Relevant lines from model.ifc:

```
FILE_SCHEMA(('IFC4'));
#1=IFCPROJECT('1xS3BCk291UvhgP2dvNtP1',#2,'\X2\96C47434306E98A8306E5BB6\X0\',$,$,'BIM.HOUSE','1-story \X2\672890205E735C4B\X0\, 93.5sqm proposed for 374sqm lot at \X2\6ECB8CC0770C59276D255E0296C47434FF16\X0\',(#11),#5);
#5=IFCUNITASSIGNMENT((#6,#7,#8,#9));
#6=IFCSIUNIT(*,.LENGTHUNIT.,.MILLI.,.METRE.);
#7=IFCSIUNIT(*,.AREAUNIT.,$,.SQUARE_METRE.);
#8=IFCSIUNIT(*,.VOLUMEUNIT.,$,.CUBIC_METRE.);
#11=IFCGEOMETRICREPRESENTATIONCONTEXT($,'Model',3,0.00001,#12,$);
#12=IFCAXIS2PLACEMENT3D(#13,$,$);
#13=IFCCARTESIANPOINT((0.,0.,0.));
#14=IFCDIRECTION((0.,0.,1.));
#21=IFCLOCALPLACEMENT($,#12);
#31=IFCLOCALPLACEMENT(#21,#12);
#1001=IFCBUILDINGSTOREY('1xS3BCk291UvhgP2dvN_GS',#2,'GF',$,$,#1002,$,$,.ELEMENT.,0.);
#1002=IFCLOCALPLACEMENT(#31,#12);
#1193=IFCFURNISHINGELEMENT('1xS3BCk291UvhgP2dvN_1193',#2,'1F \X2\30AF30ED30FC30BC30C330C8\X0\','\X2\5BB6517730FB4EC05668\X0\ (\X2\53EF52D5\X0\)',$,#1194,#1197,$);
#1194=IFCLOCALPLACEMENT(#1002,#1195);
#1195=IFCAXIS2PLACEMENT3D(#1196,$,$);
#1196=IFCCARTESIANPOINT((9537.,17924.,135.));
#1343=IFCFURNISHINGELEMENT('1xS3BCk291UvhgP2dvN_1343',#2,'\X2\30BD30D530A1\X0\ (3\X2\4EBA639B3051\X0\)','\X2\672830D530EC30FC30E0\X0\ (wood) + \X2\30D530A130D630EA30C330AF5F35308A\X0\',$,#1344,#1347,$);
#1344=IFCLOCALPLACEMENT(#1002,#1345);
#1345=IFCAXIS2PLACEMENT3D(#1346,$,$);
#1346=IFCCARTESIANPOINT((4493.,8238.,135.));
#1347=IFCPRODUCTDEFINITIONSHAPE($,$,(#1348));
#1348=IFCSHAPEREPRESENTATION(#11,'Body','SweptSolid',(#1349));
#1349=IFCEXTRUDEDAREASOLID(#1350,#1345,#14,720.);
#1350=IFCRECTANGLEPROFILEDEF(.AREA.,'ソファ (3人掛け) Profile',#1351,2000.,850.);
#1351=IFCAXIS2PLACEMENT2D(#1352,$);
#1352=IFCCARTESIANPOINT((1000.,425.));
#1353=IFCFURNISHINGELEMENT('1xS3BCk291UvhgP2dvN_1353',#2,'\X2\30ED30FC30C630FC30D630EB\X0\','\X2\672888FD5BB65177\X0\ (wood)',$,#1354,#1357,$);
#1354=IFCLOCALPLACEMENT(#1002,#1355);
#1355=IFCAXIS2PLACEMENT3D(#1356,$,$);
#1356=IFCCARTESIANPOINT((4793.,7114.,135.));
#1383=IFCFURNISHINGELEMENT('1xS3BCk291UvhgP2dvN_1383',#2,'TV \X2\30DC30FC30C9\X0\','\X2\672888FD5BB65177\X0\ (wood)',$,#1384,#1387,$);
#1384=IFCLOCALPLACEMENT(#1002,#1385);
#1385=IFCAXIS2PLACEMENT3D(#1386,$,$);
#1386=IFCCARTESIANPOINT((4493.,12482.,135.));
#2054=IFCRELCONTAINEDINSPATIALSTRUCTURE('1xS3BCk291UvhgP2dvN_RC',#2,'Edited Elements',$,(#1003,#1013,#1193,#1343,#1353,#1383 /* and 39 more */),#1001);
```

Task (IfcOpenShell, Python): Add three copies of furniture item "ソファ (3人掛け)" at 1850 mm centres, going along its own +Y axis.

```python
import ifcopenshell
import ifcopenshell.api.geometry
import ifcopenshell.api.root
import ifcopenshell.util.element
import ifcopenshell.util.placement
import ifcopenshell.util.unit

model = ifcopenshell.open("model.ifc")
unit_scale = ifcopenshell.util.unit.calculate_unit_scale(model)


def reuse_history(source, copy):
    """copy_class also copies each property set's owner history, people and application; keep the originals."""
    for rel in copy.IsDefinedBy:
        if rel.is_a("IfcRelDefinesByProperties") and (history := rel.RelatingPropertyDefinition.OwnerHistory):
            rel.RelatingPropertyDefinition.OwnerHistory = source.OwnerHistory
            ifcopenshell.util.element.remove_deep2(model, history)


source = model.by_guid("1xS3BCk291UvhgP2dvN_1343")
base = ifcopenshell.util.placement.get_local_placement(source.ObjectPlacement)
step = base[:3, 1] * 1.85 / unit_scale

for i in range(1, 4):
    copy = ifcopenshell.api.root.copy_class(model, product=source)
    copy.Representation = ifcopenshell.util.element.copy_deep(
        model, source.Representation, exclude=["IfcGeometricRepresentationContext", "IfcRepresentationMap"]
    )
    reuse_history(source, copy)
    matrix = base.copy()
    matrix[:3, 3] += i * step
    print("added at", matrix[:3, 3].round(3) + 0.0)
    ifcopenshell.api.geometry.edit_object_placement(model, product=copy, matrix=matrix, is_si=False)

model.write("model-out.ifc")
```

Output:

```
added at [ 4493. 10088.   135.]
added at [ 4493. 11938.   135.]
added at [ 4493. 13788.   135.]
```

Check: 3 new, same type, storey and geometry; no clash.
